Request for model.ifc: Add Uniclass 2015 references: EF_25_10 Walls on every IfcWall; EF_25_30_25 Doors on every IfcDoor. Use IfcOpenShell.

First a look at what the model holds.

```python
import ifcopenshell

model = ifcopenshell.open("model.ifc")
print(model.schema)
print("classifications:", [c.Name for c in model.by_type("IfcClassification")])
for ifc_class in ("IfcDoor", "IfcRoof", "IfcStair", "IfcWall", "IfcWindow"):
    print(ifc_class, len(model.by_type(ifc_class)))
```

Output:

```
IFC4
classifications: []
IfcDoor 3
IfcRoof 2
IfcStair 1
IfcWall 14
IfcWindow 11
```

```python
import ifcopenshell
import ifcopenshell.api.classification

model = ifcopenshell.open("model.ifc")

system = ifcopenshell.api.classification.add_classification(model, classification="Uniclass 2015")

codes = {
    "IfcWall": ("EF_25_10", "Walls"),
    "IfcDoor": ("EF_25_30_25", "Doors"),
}
for ifc_class, (code, name) in codes.items():
    products = model.by_type(ifc_class)
    ifcopenshell.api.classification.add_reference(
        model, products=products, classification=system, identification=code, name=name
    )
    print(code, len(products))

model.write("model_v2.ifc")
```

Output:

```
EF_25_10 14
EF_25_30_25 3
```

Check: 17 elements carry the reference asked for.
